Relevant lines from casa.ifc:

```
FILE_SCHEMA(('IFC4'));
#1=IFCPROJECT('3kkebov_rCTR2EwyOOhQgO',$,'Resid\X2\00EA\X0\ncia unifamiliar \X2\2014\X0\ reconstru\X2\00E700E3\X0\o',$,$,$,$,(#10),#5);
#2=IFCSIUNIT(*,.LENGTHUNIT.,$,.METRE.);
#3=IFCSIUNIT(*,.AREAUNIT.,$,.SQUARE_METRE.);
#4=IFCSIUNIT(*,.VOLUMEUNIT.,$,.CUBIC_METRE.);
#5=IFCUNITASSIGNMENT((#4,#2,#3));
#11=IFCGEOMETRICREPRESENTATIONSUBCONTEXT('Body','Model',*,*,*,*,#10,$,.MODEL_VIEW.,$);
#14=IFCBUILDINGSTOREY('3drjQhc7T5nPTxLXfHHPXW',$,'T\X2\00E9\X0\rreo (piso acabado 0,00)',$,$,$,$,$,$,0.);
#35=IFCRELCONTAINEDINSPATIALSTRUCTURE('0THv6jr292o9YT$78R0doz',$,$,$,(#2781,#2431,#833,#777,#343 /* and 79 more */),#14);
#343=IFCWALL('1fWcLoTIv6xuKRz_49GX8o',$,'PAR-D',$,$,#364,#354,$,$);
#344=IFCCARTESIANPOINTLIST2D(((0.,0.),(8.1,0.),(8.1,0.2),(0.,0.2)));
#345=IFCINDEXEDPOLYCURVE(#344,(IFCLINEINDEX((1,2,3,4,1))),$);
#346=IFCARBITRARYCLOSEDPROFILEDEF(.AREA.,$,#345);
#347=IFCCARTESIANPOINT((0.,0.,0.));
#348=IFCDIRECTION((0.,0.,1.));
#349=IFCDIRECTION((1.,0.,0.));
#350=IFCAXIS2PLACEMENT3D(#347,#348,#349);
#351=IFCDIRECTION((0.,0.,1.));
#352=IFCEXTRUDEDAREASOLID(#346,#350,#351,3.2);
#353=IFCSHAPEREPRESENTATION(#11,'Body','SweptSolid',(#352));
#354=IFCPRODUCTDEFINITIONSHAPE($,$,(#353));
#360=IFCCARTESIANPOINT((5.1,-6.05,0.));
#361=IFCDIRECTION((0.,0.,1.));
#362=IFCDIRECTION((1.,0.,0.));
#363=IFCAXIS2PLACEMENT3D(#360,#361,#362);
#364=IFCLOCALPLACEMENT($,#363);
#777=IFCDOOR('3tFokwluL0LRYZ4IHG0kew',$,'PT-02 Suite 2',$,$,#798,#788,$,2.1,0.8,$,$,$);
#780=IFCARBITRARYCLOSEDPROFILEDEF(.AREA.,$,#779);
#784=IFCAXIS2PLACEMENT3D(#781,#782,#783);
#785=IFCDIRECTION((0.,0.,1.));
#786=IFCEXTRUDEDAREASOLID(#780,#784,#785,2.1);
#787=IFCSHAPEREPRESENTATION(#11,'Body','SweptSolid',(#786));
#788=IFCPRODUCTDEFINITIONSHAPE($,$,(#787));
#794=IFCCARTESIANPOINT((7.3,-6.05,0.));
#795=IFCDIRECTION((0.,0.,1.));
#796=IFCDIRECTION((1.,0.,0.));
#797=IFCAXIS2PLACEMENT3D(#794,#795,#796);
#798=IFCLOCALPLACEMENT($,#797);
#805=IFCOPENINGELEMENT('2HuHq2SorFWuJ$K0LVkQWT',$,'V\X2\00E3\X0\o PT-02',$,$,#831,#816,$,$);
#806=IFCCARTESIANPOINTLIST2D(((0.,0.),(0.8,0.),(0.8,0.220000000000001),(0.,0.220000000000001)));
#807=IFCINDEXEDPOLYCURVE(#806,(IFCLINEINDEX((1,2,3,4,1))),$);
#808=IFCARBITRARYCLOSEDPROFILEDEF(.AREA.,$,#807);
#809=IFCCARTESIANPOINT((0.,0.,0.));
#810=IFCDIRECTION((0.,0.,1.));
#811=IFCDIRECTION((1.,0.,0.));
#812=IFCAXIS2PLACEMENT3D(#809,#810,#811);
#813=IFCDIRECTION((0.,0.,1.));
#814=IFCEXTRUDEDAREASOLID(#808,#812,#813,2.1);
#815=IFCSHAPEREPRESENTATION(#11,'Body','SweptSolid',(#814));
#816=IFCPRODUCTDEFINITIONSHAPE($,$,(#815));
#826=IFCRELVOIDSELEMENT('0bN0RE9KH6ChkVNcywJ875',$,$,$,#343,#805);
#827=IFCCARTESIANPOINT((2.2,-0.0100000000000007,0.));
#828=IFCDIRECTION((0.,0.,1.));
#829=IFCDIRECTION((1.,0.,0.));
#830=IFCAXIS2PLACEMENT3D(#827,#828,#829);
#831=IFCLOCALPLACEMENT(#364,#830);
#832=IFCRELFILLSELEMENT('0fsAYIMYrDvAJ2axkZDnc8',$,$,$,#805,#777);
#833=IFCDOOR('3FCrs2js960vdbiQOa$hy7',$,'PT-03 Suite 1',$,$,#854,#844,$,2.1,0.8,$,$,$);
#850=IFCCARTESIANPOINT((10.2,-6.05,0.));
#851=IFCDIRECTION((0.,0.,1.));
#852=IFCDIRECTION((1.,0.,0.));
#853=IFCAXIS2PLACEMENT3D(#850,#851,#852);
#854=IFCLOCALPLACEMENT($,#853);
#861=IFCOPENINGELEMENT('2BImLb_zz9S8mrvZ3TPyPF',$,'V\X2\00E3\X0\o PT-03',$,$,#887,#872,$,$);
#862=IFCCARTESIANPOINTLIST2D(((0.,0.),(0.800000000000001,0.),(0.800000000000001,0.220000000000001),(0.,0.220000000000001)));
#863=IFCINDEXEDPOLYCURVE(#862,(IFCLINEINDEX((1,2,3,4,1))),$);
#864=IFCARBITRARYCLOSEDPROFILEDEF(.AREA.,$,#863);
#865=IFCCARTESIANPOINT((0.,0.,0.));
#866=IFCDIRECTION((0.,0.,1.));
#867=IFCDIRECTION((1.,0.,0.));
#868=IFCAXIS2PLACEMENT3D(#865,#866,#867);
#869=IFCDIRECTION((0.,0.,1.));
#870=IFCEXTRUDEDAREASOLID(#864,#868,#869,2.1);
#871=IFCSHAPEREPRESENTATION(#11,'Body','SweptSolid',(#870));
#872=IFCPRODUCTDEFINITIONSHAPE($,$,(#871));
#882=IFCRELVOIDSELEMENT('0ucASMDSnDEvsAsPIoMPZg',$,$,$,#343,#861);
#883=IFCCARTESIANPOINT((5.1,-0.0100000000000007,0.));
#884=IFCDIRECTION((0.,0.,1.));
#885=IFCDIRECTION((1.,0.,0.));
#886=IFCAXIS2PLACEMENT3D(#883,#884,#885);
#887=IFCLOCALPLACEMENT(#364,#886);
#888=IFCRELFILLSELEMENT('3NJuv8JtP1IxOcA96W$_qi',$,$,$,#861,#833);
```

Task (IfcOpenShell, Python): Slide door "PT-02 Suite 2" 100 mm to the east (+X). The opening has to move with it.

```python
import ifcopenshell
import ifcopenshell.api.geometry
import ifcopenshell.util.placement
import ifcopenshell.util.unit

model = ifcopenshell.open("casa.ifc")
unit_scale = ifcopenshell.util.unit.calculate_unit_scale(model)

door = model.by_guid("3tFokwluL0LRYZ4IHG0kew")
opening = door.FillsVoids[0].RelatingOpeningElement
wall = opening.VoidsElements[0].RelatingBuildingElement

wall_matrix = ifcopenshell.util.placement.get_local_placement(wall.ObjectPlacement)
shift = wall_matrix[:3, 0] * 0.1 / unit_scale
before = ifcopenshell.util.placement.get_local_placement(door.ObjectPlacement)[:3, 3].copy()

# The door is not placed relative to its opening, so move both.
for product in (opening, door):
    matrix = ifcopenshell.util.placement.get_local_placement(product.ObjectPlacement)
    matrix[:3, 3] += shift
    ifcopenshell.api.geometry.edit_object_placement(model, product=product, matrix=matrix, is_si=False)

after = ifcopenshell.util.placement.get_local_placement(door.ObjectPlacement)[:3, 3]
print("door moved by", (after - before).round(3) + 0.0)

model.write("casa_v2.ifc")
```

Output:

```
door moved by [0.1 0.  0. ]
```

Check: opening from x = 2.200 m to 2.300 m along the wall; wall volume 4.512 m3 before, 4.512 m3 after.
